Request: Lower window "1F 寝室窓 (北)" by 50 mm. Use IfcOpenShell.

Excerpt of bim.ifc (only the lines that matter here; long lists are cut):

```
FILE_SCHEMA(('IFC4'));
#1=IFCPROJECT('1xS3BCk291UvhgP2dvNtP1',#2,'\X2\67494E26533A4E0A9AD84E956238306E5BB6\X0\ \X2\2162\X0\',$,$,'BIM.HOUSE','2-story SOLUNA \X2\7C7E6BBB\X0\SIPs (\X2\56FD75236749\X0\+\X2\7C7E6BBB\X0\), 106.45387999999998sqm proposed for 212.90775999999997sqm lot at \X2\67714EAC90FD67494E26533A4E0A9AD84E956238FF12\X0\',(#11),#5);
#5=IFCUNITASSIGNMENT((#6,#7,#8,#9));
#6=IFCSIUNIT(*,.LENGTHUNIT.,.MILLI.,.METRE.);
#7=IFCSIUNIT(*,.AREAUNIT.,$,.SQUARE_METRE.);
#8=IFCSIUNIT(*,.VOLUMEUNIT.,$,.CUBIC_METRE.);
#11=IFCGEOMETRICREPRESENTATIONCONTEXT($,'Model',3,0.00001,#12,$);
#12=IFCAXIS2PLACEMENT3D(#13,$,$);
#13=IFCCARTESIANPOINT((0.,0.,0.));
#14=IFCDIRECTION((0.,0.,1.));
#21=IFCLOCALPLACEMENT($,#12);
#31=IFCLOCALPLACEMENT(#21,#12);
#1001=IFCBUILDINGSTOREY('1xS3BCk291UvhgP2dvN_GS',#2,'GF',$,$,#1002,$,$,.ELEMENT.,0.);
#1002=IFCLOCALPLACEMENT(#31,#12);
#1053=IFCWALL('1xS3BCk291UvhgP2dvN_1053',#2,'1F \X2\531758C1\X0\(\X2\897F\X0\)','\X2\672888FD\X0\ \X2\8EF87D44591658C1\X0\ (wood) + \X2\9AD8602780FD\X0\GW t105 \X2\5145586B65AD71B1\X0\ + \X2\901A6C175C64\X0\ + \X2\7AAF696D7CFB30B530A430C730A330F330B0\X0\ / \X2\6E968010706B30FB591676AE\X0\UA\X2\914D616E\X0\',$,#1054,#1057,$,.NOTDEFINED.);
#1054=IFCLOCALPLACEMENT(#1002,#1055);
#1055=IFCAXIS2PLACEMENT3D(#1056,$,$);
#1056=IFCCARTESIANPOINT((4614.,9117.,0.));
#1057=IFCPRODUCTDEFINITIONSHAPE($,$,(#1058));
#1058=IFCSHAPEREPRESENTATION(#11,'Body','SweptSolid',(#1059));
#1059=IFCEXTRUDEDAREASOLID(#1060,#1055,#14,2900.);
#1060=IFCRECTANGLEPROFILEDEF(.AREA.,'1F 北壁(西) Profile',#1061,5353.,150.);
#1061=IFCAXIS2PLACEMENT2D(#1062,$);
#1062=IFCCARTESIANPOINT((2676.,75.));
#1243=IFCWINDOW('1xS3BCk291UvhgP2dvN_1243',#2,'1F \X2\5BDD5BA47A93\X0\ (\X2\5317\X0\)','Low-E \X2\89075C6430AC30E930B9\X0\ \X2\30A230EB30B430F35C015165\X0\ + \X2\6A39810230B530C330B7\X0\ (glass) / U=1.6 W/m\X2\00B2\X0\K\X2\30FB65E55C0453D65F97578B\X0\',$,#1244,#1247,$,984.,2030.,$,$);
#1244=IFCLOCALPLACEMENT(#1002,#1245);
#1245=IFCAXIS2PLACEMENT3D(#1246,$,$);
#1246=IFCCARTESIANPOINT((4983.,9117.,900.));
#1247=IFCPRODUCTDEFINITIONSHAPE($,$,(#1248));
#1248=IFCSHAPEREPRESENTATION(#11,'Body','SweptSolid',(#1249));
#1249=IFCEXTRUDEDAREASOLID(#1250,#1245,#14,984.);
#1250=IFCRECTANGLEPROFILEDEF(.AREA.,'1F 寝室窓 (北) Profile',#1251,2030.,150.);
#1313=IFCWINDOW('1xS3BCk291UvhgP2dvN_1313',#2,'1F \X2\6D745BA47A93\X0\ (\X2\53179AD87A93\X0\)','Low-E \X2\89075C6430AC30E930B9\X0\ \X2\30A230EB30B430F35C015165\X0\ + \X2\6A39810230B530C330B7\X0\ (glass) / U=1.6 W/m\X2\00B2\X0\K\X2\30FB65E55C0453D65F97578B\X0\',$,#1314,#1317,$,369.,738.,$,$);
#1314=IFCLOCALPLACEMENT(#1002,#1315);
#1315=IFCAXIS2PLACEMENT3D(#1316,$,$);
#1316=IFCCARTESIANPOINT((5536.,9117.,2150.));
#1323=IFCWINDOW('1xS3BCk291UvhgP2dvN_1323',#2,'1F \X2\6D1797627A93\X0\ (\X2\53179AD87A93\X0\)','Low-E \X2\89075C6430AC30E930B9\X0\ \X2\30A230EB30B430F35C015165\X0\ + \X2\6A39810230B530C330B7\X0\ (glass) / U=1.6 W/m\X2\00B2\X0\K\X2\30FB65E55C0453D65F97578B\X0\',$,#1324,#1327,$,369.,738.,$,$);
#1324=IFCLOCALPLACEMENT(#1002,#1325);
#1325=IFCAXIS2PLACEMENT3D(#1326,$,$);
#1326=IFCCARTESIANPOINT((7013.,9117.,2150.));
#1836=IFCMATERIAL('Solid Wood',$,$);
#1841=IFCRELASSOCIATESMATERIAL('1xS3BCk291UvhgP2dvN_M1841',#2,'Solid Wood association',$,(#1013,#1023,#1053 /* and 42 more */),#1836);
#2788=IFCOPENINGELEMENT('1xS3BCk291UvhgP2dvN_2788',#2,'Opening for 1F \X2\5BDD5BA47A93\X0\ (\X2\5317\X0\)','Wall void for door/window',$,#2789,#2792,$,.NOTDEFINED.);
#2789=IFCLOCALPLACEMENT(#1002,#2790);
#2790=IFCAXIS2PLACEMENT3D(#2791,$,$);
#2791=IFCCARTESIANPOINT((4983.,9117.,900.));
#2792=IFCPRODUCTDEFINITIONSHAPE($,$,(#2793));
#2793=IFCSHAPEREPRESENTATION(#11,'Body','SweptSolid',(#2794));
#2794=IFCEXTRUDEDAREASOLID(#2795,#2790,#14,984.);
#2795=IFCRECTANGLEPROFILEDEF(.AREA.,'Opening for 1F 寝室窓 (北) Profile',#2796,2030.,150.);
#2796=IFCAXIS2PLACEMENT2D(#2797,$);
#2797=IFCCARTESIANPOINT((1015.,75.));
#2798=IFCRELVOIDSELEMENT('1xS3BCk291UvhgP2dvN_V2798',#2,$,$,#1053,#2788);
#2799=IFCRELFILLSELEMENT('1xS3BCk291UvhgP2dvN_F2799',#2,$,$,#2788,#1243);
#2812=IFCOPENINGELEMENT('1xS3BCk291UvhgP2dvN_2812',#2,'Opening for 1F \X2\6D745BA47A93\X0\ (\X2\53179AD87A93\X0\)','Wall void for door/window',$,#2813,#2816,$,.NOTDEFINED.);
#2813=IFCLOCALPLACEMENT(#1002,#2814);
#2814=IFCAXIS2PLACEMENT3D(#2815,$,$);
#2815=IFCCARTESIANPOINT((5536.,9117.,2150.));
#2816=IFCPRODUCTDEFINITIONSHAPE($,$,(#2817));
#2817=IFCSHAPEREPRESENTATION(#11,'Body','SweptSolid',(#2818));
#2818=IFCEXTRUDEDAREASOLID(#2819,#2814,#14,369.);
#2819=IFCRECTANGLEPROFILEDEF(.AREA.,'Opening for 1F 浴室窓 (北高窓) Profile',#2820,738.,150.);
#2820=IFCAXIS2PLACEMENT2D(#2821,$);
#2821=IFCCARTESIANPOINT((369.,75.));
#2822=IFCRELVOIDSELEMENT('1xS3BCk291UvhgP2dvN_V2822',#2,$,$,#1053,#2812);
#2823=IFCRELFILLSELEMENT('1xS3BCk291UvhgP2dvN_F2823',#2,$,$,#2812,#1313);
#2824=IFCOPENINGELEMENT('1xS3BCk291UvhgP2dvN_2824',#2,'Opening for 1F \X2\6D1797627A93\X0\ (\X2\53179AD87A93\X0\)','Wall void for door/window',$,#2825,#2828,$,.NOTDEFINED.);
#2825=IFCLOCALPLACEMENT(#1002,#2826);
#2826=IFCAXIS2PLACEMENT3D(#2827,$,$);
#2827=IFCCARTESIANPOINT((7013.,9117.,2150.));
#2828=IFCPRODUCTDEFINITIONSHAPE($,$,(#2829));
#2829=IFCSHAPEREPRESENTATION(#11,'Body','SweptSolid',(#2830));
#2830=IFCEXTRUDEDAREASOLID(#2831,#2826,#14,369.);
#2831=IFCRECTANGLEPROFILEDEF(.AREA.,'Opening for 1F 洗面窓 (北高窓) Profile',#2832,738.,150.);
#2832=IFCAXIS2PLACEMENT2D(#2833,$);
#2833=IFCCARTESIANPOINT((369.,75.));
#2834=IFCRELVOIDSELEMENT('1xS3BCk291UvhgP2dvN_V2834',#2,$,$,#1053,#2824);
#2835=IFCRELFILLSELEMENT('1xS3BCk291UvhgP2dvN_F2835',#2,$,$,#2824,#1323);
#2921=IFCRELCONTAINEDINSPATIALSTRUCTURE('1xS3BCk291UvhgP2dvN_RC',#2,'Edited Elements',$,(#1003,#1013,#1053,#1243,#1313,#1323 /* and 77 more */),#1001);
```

```python
import numpy as np
import ifcopenshell
import ifcopenshell.api.geometry
import ifcopenshell.util.placement
import ifcopenshell.util.unit

model = ifcopenshell.open("bim.ifc")
unit_scale = ifcopenshell.util.unit.calculate_unit_scale(model)

window = model.by_guid("1xS3BCk291UvhgP2dvN_1243")
opening = window.FillsVoids[0].RelatingOpeningElement
dz = -0.05 / unit_scale

shift = np.array([0.0, 0.0, dz])
# The window is not placed relative to its opening, so move both.
for product in (opening, window):
    matrix = ifcopenshell.util.placement.get_local_placement(product.ObjectPlacement)
    matrix[:3, 3] += shift
    ifcopenshell.api.geometry.edit_object_placement(model, product=product, matrix=matrix, is_si=False)

print(f"moved by {dz * unit_scale:+.3f} m")

model.write("bim_rev.ifc")
```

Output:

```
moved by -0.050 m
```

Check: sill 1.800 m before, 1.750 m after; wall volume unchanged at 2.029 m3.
